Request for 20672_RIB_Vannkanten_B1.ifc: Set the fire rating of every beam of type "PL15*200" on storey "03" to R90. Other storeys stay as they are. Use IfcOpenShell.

First a look at what the model holds.

```python
import ifcopenshell
import ifcopenshell.util.element

model = ifcopenshell.open("20672_RIB_Vannkanten_B1.ifc")
print(model.schema)
storey = next(s for s in model.by_type("IfcBuildingStorey") if s.Name == "03")
beams = [e for e in ifcopenshell.util.element.get_decomposition(storey) if e.is_a("IfcBeam")]
seen = {}
for e in beams:
    element_type = ifcopenshell.util.element.get_type(e)
    key = (element_type.Name if element_type != e and element_type else None, ifcopenshell.util.element.get_pset(e, "Pset_BeamCommon", "FireRating"))
    seen[key] = seen.get(key, 0) + 1
for (name, value), count in sorted(seen.items(), key=str):
    print(count, "x", name, "|", value)
```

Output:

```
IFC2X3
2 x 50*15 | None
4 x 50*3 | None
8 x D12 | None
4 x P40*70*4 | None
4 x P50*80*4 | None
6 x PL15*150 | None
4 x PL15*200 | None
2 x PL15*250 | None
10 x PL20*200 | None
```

```python
import ifcopenshell
import ifcopenshell.api.pset
import ifcopenshell.util.element

model = ifcopenshell.open("20672_RIB_Vannkanten_B1.ifc")

storey = next(s for s in model.by_type("IfcBuildingStorey") if s.Name == "03")
beams = [e for e in ifcopenshell.util.element.get_decomposition(storey) if e.is_a("IfcBeam")]

count = 0
for e in beams:
    element_type = ifcopenshell.util.element.get_type(e)
    if element_type in (None, e) or element_type.Name != "PL15*200":
        continue
    # add_pset returns the element's existing set when there is one.
    pset = ifcopenshell.api.pset.add_pset(model, product=e, name="Pset_BeamCommon")
    ifcopenshell.api.pset.edit_pset(model, pset=pset, properties={"FireRating": "R90"})
    count += 1

print(count, "beams updated")

model.write("20672_RIB_Vannkanten_B1-out.ifc")
```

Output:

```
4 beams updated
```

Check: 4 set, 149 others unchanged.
